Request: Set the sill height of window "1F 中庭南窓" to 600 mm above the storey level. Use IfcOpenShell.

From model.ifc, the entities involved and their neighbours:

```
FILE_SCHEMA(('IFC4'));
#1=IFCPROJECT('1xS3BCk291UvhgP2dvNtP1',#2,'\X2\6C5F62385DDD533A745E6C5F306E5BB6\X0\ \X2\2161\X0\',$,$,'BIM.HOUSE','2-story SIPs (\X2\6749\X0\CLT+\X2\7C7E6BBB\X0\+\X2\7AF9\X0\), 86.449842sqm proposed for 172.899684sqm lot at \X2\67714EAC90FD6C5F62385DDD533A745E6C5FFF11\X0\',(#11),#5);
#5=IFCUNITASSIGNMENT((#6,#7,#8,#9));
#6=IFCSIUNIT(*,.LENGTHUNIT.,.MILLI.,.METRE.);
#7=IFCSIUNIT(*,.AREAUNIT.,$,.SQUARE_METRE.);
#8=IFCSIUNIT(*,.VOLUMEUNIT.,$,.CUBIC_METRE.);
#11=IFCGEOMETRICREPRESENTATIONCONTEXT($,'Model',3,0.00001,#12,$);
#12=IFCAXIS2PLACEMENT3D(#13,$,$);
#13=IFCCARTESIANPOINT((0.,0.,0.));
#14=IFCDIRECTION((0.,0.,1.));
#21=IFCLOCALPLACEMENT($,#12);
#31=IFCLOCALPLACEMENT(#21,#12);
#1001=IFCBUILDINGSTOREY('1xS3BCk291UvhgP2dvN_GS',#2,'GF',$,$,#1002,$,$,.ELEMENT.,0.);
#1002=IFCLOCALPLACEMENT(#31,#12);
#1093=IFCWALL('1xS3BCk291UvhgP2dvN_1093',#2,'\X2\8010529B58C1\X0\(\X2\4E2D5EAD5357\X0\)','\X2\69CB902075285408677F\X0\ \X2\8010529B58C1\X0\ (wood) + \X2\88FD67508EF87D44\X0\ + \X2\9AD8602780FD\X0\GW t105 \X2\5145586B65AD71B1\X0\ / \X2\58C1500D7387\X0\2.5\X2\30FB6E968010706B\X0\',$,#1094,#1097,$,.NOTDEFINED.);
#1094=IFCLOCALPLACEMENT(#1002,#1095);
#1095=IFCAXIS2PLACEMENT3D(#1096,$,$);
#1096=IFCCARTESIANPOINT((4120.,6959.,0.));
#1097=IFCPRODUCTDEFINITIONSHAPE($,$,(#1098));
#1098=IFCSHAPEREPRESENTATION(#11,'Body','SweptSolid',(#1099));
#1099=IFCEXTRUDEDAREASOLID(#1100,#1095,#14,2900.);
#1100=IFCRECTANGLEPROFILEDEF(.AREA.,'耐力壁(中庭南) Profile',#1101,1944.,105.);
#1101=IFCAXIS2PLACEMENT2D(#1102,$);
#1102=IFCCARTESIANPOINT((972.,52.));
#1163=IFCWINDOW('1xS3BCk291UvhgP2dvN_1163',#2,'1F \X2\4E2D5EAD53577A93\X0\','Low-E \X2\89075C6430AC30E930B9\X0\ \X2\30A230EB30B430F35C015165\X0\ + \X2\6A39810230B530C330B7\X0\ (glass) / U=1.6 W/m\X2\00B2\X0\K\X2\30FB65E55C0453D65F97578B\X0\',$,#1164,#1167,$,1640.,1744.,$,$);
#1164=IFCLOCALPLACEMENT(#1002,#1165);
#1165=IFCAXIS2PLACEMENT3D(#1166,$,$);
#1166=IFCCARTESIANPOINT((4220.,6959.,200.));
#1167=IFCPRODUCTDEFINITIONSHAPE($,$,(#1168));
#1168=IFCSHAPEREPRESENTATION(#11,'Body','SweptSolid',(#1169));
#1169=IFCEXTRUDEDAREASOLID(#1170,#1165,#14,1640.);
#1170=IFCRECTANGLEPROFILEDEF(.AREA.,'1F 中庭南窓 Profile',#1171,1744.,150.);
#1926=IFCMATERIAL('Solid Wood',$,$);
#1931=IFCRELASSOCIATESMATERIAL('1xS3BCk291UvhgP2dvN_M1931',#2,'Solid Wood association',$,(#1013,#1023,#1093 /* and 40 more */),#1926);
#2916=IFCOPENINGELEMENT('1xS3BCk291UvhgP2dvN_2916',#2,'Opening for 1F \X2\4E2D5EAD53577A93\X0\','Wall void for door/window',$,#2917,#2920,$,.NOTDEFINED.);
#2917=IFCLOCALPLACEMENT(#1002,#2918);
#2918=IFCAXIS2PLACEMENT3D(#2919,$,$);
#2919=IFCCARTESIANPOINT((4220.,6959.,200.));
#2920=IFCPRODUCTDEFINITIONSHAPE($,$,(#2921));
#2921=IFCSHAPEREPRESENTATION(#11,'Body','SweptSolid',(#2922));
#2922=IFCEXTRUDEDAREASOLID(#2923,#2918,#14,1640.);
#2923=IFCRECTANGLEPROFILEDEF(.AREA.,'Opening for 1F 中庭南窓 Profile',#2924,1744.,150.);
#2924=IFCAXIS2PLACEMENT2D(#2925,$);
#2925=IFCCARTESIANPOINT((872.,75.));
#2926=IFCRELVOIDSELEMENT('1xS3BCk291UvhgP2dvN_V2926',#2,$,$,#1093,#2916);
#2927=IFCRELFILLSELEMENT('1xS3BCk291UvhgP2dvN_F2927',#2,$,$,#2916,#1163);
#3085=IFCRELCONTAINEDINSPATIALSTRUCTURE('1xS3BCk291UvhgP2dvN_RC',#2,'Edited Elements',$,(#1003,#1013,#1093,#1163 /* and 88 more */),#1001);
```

```python
import numpy as np
import ifcopenshell
import ifcopenshell.api.geometry
import ifcopenshell.geom
import ifcopenshell.util.element
import ifcopenshell.util.placement
import ifcopenshell.util.shape
import ifcopenshell.util.unit

model = ifcopenshell.open("model.ifc")
unit_scale = ifcopenshell.util.unit.calculate_unit_scale(model)

window = model.by_id(1163)
opening = window.FillsVoids[0].RelatingOpeningElement
storey = ifcopenshell.util.element.get_container(window, ifc_class="IfcBuildingStorey")
level = ifcopenshell.util.placement.get_local_placement(storey.ObjectPlacement)[2, 3]

# The opening's origin need not be at the sill, so measure its lowest point.
shape = ifcopenshell.geom.create_shape(ifcopenshell.geom.settings(), opening)
bottom = ifcopenshell.util.shape.get_shape_bottom_elevation(shape, shape.geometry) / unit_scale
dz = level + 0.6 / unit_scale - bottom

shift = np.array([0.0, 0.0, dz])
# The window is not placed relative to its opening, so move both.
for product in (opening, window):
    matrix = ifcopenshell.util.placement.get_local_placement(product.ObjectPlacement)
    matrix[:3, 3] += shift
    ifcopenshell.api.geometry.edit_object_placement(model, product=product, matrix=matrix, is_si=False)

print(f"moved by {dz * unit_scale:+.3f} m")

model.write("model_updated.ifc")
```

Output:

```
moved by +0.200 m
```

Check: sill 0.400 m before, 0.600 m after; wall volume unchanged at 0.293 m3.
